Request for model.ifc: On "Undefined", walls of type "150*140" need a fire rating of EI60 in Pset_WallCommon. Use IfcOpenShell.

First a look at what the model holds.

```python
import ifcopenshell
import ifcopenshell.util.element

model = ifcopenshell.open("model.ifc")
print(model.schema)
storey = next(s for s in model.by_type("IfcBuildingStorey") if s.Name == "Undefined")
walls = [e for e in ifcopenshell.util.element.get_decomposition(storey) if e.is_a("IfcWall")]
seen = {}
for e in walls:
    element_type = ifcopenshell.util.element.get_type(e)
    key = (element_type.Name if element_type != e and element_type else None, ifcopenshell.util.element.get_pset(e, "Pset_WallCommon", "FireRating"))
    seen[key] = seen.get(key, 0) + 1
for (name, value), count in sorted(seen.items(), key=str):
    print(count, "x", name, "|", value)
```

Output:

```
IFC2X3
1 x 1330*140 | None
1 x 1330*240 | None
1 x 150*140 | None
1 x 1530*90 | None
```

```python
import ifcopenshell
import ifcopenshell.api.pset
import ifcopenshell.util.element

model = ifcopenshell.open("model.ifc")

storey = next(s for s in model.by_type("IfcBuildingStorey") if s.Name == "Undefined")
walls = [e for e in ifcopenshell.util.element.get_decomposition(storey) if e.is_a("IfcWall")]

count = 0
for e in walls:
    element_type = ifcopenshell.util.element.get_type(e)
    if element_type in (None, e) or element_type.Name != "150*140":
        continue
    # add_pset returns the element's existing set when there is one.
    pset = ifcopenshell.api.pset.add_pset(model, product=e, name="Pset_WallCommon")
    ifcopenshell.api.pset.edit_pset(model, pset=pset, properties={"FireRating": "EI60"})
    count += 1

print(count, "walls updated")

model.write("model_updated.ifc")
```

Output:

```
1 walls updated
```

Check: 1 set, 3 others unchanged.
